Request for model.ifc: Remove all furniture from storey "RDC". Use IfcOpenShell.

First a look at what the model holds.

```python
import ifcopenshell
import ifcopenshell.util.element

model = ifcopenshell.open("model.ifc")
print(model.schema)
storey = next(s for s in model.by_type("IfcBuildingStorey") if s.Name == "RDC")
furniture = [e for e in ifcopenshell.util.element.get_decomposition(storey) if e.is_a("IfcFurnishingElement")]
seen = {}
for e in furniture:
    element_type = ifcopenshell.util.element.get_type(e)
    name = element_type.Name if element_type not in (None, e) else None
    seen[name] = seen.get(name, 0) + 1
for name, count in sorted(seen.items(), key=str):
    print(count, "x", name)
```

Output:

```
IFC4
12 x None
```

```python
import ifcopenshell
import ifcopenshell.api.root
import ifcopenshell.util.element

model = ifcopenshell.open("model.ifc")

storey = next(s for s in model.by_type("IfcBuildingStorey") if s.Name == "RDC")
furniture = [e for e in ifcopenshell.util.element.get_decomposition(storey) if e.is_a("IfcFurnishingElement")]

for e in furniture:
    ifcopenshell.api.root.remove_product(model, product=e)
print(len(furniture), "removed")

model.write("model_edited.ifc")
```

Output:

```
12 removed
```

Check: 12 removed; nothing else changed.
